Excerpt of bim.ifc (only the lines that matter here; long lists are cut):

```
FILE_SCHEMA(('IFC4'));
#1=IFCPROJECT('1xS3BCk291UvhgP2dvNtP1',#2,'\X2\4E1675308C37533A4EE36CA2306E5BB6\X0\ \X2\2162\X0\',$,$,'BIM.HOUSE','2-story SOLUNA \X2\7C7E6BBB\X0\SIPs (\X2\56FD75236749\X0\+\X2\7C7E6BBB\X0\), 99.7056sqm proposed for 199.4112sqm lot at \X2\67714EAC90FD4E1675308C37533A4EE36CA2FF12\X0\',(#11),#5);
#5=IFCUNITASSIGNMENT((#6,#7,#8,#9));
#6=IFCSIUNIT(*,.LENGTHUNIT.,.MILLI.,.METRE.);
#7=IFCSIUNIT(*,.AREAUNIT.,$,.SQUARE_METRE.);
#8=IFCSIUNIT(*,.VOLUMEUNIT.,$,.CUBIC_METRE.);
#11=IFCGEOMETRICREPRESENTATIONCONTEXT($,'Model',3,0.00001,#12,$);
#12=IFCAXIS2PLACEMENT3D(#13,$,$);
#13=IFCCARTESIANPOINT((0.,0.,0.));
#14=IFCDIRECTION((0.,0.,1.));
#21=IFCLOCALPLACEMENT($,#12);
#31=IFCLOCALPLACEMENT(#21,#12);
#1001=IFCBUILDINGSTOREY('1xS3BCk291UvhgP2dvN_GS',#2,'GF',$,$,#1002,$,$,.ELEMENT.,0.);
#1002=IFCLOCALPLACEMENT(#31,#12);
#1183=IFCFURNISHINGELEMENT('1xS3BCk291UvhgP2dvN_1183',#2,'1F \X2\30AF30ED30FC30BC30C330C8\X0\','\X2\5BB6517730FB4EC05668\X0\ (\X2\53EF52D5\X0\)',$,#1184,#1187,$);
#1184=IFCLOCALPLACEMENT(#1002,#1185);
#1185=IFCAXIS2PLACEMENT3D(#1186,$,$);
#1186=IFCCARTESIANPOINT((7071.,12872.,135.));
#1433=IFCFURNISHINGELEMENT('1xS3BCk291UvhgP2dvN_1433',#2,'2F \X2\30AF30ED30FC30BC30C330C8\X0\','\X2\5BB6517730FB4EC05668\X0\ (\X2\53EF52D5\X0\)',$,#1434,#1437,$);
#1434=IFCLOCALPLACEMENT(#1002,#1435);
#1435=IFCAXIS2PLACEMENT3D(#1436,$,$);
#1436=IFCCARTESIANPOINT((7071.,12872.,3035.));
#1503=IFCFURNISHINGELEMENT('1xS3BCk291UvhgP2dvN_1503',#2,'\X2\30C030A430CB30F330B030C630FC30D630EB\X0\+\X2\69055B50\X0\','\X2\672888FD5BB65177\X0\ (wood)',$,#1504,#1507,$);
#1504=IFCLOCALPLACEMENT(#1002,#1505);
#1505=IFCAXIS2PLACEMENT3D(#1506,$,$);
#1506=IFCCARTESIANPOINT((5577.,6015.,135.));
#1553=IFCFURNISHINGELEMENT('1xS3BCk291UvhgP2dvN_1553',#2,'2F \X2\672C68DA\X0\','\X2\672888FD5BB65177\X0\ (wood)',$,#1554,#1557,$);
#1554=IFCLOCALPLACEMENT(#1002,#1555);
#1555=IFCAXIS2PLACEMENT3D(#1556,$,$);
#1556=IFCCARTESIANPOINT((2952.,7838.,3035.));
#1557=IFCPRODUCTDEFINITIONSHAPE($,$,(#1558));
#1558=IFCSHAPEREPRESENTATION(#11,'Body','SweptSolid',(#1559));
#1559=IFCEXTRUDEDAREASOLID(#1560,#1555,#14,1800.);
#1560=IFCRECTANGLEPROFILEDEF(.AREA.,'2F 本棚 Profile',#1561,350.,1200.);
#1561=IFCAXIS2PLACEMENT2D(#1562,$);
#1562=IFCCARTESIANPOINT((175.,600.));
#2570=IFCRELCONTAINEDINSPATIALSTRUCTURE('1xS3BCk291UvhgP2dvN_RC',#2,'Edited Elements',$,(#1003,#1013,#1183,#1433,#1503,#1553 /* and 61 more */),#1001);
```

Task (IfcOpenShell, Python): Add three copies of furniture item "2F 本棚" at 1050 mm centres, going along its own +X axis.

```python
import ifcopenshell
import ifcopenshell.api.geometry
import ifcopenshell.api.root
import ifcopenshell.util.element
import ifcopenshell.util.placement
import ifcopenshell.util.unit

model = ifcopenshell.open("bim.ifc")
unit_scale = ifcopenshell.util.unit.calculate_unit_scale(model)


def reuse_history(source, copy):
    """copy_class also copies each property set's owner history, people and application; keep the originals."""
    for rel in copy.IsDefinedBy:
        if rel.is_a("IfcRelDefinesByProperties") and (history := rel.RelatingPropertyDefinition.OwnerHistory):
            rel.RelatingPropertyDefinition.OwnerHistory = source.OwnerHistory
            ifcopenshell.util.element.remove_deep2(model, history)


source = model.by_guid("1xS3BCk291UvhgP2dvN_1553")
base = ifcopenshell.util.placement.get_local_placement(source.ObjectPlacement)
step = base[:3, 0] * 1.05 / unit_scale

for i in range(1, 4):
    copy = ifcopenshell.api.root.copy_class(model, product=source)
    copy.Representation = ifcopenshell.util.element.copy_deep(
        model, source.Representation, exclude=["IfcGeometricRepresentationContext", "IfcRepresentationMap"]
    )
    reuse_history(source, copy)
    matrix = base.copy()
    matrix[:3, 3] += i * step
    print("added at", matrix[:3, 3].round(3) + 0.0)
    ifcopenshell.api.geometry.edit_object_placement(model, product=copy, matrix=matrix, is_si=False)

model.write("bim_v2.ifc")
```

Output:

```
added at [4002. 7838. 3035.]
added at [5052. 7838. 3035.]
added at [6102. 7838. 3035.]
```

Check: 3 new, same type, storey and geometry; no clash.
